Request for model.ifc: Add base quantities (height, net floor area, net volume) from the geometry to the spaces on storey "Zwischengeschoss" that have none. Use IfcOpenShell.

First a look at what the model holds.

```python
import ifcopenshell
import ifcopenshell.util.element
import ifcopenshell.util.unit

model = ifcopenshell.open("model.ifc")
print(model.schema)
for unit_type in ("LENGTHUNIT", "AREAUNIT", "VOLUMEUNIT"):
    print(unit_type, ifcopenshell.util.unit.calculate_unit_scale(model, unit_type))
storey = next(s for s in model.by_type("IfcBuildingStorey") if s.Name == "Zwischengeschoss")
spaces = [e for e in ifcopenshell.util.element.get_decomposition(storey) if e.is_a("IfcSpace")]
for e in sorted(spaces, key=lambda e: e.id()):
    print(e.id(), e.is_a(), e.Name, list(ifcopenshell.util.element.get_psets(e, qtos_only=True)), sep=" | ")
```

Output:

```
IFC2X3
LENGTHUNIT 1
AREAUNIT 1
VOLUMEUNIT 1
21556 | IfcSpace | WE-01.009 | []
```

```python
import ifcopenshell
import ifcopenshell.api.pset
import ifcopenshell.geom
import ifcopenshell.util.element
import ifcopenshell.util.shape
import ifcopenshell.util.unit

model = ifcopenshell.open("model.ifc")
unit_scale = ifcopenshell.util.unit.calculate_unit_scale(model)
area_scale = ifcopenshell.util.unit.calculate_unit_scale(model, "AREAUNIT")
volume_scale = ifcopenshell.util.unit.calculate_unit_scale(model, "VOLUMEUNIT")
settings = ifcopenshell.geom.settings()

storey = next(s for s in model.by_type("IfcBuildingStorey") if s.Name == "Zwischengeschoss")
spaces = [e for e in ifcopenshell.util.element.get_decomposition(storey) if e.is_a("IfcSpace")]

for e in sorted(spaces, key=lambda e: e.id()):
    if ifcopenshell.util.element.get_psets(e, qtos_only=True, should_inherit=False):
        continue
    # Geometry comes back in metres, in the element's own axes.
    shape = ifcopenshell.geom.create_shape(settings, e)
    values = {
        "Height": ifcopenshell.util.shape.get_z(shape.geometry) / unit_scale,
        "NetFloorArea": ifcopenshell.util.shape.get_footprint_area(shape.geometry) / area_scale,
        "NetVolume": ifcopenshell.util.shape.get_volume(shape.geometry) / volume_scale,
    }
    qto = ifcopenshell.api.pset.add_qto(model, product=e, name="BaseQuantities")
    ifcopenshell.api.pset.edit_qto(model, qto=qto, properties=values)
    print(e.id(), {k: round(v, 3) for k, v in values.items()})

model.write("model-out.ifc")
```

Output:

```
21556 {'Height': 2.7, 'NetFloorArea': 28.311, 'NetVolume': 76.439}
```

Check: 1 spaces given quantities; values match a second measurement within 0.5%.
